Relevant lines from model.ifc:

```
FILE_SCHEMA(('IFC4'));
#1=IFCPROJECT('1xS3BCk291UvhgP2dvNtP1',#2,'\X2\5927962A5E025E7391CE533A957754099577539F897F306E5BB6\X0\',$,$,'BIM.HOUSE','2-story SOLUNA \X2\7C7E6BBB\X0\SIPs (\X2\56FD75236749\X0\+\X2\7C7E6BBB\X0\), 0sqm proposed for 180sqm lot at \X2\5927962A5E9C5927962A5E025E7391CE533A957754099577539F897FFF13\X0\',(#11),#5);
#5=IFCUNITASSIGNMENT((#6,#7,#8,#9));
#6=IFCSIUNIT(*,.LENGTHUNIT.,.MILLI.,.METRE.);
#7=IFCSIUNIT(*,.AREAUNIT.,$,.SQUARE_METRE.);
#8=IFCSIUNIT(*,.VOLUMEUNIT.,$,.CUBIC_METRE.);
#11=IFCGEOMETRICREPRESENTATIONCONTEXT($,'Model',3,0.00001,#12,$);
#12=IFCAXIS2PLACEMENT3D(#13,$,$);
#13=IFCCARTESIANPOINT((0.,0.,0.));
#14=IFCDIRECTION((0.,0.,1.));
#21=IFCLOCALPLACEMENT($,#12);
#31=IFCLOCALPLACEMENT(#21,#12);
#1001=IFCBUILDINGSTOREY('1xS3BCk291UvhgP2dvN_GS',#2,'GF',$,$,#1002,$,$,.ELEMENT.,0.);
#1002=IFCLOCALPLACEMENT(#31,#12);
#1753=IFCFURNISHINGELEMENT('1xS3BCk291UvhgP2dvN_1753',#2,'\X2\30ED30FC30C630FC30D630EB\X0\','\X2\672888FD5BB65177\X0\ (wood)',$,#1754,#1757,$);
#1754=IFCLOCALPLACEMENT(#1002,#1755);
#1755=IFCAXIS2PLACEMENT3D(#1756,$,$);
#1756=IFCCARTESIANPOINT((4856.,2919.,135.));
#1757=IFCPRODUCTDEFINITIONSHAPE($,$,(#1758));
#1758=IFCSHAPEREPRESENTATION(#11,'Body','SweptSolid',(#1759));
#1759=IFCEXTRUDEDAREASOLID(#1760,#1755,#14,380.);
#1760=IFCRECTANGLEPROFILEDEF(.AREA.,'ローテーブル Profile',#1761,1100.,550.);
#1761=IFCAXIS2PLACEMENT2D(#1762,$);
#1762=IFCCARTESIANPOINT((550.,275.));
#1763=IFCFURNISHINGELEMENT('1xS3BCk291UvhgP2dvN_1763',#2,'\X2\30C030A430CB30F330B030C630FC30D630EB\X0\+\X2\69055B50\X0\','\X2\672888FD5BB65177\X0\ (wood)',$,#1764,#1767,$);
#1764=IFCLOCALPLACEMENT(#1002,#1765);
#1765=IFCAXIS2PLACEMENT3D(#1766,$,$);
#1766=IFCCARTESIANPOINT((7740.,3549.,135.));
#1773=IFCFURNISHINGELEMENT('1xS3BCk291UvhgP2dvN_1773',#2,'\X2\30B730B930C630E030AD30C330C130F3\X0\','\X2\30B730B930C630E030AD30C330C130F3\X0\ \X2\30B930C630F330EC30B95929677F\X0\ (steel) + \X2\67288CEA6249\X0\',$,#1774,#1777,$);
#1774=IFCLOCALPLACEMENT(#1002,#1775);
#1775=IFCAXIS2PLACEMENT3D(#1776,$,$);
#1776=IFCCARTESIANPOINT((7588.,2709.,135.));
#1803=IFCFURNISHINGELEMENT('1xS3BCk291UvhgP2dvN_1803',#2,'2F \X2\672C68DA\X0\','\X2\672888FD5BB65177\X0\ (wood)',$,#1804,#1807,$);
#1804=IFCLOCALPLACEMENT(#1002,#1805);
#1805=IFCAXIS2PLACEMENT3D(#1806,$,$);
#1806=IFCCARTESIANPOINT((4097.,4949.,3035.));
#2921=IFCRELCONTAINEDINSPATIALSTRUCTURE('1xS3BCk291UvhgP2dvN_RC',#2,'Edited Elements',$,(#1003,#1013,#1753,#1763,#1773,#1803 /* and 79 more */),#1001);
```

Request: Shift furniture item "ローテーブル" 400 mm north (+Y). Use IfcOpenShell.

```python
import ifcopenshell
import ifcopenshell.api.geometry
import ifcopenshell.util.placement
import ifcopenshell.util.unit

model = ifcopenshell.open("model.ifc")
unit_scale = ifcopenshell.util.unit.calculate_unit_scale(model)

item = model.by_guid("1xS3BCk291UvhgP2dvN_1753")
matrix = ifcopenshell.util.placement.get_local_placement(item.ObjectPlacement)
matrix[1, 3] += 0.4 / unit_scale
ifcopenshell.api.geometry.edit_object_placement(model, product=item, matrix=matrix, is_si=False)

print(ifcopenshell.util.placement.get_local_placement(item.ObjectPlacement).round(3) + 0.0)

model.write("model-out.ifc")
```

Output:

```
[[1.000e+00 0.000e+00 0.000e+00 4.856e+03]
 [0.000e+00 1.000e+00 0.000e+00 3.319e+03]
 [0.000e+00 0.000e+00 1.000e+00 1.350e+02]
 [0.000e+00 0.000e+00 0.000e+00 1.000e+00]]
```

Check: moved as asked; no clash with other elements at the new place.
